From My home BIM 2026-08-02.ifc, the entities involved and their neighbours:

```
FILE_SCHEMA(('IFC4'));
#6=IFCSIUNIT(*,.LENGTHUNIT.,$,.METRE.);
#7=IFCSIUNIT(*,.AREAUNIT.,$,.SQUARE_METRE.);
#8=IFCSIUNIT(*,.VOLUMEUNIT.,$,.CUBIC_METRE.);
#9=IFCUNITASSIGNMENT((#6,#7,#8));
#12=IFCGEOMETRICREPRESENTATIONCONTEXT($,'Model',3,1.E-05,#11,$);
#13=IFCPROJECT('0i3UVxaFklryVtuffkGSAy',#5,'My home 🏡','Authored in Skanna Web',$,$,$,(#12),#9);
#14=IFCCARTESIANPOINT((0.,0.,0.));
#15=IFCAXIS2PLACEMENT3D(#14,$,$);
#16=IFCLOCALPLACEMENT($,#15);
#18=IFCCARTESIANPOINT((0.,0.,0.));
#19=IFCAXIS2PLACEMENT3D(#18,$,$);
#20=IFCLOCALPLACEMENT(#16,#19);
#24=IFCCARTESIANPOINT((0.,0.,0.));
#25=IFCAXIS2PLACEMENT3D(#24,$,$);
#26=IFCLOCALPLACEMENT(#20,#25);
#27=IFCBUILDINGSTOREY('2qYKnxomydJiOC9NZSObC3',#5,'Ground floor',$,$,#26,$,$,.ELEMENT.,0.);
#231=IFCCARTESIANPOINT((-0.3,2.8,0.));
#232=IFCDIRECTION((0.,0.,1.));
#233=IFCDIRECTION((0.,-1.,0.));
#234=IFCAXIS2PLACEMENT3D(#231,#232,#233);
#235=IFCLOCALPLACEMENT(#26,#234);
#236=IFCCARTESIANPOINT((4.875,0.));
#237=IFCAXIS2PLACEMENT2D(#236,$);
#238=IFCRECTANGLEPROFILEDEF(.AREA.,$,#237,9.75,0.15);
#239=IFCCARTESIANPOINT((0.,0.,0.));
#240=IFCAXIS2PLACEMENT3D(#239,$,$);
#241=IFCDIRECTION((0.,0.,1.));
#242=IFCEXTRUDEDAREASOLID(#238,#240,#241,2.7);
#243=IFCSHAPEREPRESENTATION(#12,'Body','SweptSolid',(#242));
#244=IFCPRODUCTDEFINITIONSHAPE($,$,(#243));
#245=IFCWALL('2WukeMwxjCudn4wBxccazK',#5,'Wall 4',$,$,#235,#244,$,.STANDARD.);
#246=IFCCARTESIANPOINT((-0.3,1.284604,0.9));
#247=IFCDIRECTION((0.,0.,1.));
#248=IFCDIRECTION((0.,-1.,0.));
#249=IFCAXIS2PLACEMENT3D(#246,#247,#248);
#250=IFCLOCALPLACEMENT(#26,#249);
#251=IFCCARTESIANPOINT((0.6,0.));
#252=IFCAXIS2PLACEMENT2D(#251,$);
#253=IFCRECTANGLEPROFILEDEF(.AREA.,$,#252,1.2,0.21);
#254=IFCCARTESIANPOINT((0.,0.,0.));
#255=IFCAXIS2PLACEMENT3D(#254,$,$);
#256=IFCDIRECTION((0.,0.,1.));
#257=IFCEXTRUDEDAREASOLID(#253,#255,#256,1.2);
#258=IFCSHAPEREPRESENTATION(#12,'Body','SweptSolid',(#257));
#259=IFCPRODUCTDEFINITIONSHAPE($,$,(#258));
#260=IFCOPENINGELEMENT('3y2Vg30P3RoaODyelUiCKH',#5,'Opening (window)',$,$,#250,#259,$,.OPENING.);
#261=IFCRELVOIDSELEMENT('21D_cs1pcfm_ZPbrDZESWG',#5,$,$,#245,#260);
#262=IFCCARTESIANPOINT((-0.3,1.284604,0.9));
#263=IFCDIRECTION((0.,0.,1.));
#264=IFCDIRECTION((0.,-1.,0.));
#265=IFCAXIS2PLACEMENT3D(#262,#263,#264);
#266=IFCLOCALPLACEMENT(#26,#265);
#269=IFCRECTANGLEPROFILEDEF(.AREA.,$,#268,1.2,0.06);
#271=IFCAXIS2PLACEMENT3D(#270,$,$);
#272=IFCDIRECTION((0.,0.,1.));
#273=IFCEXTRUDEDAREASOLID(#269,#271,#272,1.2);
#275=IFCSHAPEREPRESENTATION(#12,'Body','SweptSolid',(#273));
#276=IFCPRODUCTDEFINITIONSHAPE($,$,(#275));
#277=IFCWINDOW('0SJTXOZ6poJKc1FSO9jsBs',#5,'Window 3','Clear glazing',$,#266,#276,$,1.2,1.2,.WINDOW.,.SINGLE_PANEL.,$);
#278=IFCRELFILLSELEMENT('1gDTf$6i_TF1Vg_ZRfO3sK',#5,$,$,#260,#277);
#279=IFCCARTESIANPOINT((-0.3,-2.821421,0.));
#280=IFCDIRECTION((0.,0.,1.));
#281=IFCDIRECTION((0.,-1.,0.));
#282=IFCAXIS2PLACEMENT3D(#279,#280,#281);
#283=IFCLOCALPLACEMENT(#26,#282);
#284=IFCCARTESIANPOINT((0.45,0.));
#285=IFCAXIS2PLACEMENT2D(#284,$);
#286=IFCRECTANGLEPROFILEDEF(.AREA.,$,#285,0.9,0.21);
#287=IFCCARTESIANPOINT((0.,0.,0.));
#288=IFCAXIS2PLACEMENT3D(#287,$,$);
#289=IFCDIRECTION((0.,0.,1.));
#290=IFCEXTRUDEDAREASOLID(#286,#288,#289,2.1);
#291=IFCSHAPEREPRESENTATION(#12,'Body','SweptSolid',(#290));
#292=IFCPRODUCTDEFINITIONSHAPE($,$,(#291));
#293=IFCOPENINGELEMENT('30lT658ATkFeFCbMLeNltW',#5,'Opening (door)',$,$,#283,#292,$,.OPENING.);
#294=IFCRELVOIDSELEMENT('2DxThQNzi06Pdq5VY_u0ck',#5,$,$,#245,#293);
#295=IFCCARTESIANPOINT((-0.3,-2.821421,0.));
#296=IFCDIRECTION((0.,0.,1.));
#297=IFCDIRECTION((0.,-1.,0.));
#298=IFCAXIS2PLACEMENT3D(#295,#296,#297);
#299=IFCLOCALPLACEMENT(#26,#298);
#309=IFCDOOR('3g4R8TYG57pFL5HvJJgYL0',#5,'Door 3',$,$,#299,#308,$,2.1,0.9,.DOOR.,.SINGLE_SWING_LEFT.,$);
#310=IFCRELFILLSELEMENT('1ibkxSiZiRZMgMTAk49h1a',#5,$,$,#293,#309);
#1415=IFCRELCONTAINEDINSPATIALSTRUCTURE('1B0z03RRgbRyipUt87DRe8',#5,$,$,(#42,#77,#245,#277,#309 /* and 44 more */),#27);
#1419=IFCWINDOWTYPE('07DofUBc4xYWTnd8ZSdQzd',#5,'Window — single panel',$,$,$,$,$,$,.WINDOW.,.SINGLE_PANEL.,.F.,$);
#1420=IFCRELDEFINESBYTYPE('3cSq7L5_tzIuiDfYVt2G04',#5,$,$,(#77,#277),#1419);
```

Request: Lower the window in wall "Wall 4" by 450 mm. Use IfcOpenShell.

```python
import numpy as np
import ifcopenshell
import ifcopenshell.api.geometry
import ifcopenshell.util.placement
import ifcopenshell.util.unit

model = ifcopenshell.open("My home BIM 2026-08-02.ifc")
unit_scale = ifcopenshell.util.unit.calculate_unit_scale(model)

window = model.by_guid("0SJTXOZ6poJKc1FSO9jsBs")
opening = window.FillsVoids[0].RelatingOpeningElement
dz = -0.45

shift = np.array([0.0, 0.0, dz])
# The window is not placed relative to its opening, so move both.
for product in (opening, window):
    matrix = ifcopenshell.util.placement.get_local_placement(product.ObjectPlacement)
    matrix[:3, 3] += shift
    ifcopenshell.api.geometry.edit_object_placement(model, product=product, matrix=matrix, is_si=False)

print(f"moved by {dz * unit_scale:+.3f} m")

model.write("My home BIM 2026-08-02-out.ifc")
```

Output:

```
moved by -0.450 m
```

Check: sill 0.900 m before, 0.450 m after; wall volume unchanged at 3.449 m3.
